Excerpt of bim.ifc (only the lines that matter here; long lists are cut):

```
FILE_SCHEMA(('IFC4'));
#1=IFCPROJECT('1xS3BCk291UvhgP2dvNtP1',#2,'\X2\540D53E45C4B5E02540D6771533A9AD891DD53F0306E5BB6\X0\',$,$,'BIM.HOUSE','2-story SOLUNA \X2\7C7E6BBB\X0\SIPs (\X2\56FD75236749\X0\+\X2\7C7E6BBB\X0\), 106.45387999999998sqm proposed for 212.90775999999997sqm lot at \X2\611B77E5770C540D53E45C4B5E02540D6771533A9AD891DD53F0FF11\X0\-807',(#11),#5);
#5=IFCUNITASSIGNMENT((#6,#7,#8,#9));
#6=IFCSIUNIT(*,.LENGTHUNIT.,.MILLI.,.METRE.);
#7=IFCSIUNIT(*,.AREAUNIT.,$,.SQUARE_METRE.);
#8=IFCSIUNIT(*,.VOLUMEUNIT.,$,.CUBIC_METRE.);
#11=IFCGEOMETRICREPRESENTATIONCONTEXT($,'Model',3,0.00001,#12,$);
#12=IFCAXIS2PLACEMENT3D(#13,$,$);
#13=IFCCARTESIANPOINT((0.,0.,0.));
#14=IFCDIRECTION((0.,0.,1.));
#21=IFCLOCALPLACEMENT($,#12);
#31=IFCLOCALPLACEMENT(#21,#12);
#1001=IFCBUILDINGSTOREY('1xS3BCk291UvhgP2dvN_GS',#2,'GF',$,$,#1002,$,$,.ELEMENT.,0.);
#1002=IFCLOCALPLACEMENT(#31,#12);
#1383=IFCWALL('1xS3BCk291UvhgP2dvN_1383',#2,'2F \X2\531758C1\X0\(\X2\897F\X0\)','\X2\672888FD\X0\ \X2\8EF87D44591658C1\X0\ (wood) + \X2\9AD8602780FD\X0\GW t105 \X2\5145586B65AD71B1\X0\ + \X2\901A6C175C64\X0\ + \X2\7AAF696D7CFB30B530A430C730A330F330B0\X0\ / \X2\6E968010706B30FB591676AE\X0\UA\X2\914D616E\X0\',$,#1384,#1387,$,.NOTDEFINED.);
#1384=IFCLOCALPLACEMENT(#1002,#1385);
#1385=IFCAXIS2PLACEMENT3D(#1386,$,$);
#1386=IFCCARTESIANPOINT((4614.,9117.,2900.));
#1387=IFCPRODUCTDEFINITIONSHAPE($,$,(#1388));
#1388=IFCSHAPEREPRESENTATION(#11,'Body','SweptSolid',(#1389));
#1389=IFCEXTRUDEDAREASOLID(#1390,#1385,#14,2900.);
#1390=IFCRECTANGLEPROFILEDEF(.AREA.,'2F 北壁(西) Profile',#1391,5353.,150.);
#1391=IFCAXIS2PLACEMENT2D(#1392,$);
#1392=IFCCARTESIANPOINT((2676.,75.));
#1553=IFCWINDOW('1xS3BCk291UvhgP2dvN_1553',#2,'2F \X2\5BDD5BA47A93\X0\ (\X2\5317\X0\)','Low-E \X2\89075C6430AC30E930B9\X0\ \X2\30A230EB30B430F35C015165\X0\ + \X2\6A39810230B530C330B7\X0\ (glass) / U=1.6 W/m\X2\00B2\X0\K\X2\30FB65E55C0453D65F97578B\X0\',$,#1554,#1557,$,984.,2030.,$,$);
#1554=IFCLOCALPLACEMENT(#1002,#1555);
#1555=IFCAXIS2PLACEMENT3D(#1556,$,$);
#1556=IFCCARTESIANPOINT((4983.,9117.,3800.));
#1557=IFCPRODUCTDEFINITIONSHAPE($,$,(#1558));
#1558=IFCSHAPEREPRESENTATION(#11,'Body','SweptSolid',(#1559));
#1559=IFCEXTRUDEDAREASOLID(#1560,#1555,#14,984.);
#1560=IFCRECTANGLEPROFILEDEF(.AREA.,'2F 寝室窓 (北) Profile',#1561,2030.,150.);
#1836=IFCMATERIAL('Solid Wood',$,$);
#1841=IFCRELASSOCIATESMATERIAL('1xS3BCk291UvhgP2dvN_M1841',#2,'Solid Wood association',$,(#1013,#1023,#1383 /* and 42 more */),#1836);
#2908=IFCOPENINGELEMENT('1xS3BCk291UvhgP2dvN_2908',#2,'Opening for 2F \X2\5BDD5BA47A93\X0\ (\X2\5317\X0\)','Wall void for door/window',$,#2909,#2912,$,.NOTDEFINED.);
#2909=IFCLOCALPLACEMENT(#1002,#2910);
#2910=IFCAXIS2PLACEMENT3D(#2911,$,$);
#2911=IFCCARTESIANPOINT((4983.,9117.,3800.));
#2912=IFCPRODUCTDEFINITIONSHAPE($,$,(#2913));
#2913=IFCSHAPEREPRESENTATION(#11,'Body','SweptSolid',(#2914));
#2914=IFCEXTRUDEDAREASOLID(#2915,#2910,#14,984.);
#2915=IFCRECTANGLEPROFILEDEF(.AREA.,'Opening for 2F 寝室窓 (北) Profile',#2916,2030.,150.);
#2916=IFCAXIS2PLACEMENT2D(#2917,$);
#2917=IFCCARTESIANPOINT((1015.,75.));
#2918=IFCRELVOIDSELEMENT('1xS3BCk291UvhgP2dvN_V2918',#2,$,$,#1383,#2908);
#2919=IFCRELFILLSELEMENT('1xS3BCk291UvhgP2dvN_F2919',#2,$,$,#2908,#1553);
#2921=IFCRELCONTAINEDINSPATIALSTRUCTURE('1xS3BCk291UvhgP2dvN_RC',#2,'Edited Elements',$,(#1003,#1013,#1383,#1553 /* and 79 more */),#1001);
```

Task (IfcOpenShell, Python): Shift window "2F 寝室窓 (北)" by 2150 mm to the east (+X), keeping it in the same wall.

```python
import ifcopenshell
import ifcopenshell.api.geometry
import ifcopenshell.util.placement
import ifcopenshell.util.unit

model = ifcopenshell.open("bim.ifc")
unit_scale = ifcopenshell.util.unit.calculate_unit_scale(model)

window = model.by_guid("1xS3BCk291UvhgP2dvN_1553")
opening = window.FillsVoids[0].RelatingOpeningElement
wall = opening.VoidsElements[0].RelatingBuildingElement

wall_matrix = ifcopenshell.util.placement.get_local_placement(wall.ObjectPlacement)
shift = wall_matrix[:3, 0] * 2.15 / unit_scale
before = ifcopenshell.util.placement.get_local_placement(window.ObjectPlacement)[:3, 3].copy()

# The window is not placed relative to its opening, so move both.
for product in (opening, window):
    matrix = ifcopenshell.util.placement.get_local_placement(product.ObjectPlacement)
    matrix[:3, 3] += shift
    ifcopenshell.api.geometry.edit_object_placement(model, product=product, matrix=matrix, is_si=False)

after = ifcopenshell.util.placement.get_local_placement(window.ObjectPlacement)[:3, 3]
print("window moved by", (after - before).round(3) + 0.0)

model.write("bim_updated.ifc")
```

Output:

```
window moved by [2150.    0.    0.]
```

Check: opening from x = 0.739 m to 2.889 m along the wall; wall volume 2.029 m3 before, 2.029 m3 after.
